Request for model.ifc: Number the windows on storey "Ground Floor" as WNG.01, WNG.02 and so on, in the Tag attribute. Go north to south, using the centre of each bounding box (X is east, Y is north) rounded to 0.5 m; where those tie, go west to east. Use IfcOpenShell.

First a look at what the model holds.

```python
import ifcopenshell
import ifcopenshell.util.element
import ifcopenshell.util.placement

model = ifcopenshell.open("model.ifc")
print(model.schema)
storey = next(s for s in model.by_type("IfcBuildingStorey") if s.Name == "Ground Floor")
windows = [e for e in ifcopenshell.util.element.get_decomposition(storey) if e.is_a("IfcWindow")]
for e in sorted(windows, key=lambda e: e.id()):
    origin = ifcopenshell.util.placement.get_local_placement(e.ObjectPlacement)[:3, 3]
    print(e.id(), e.Tag, e.Name, origin.round(2) + 0.0, sep=" | ")
```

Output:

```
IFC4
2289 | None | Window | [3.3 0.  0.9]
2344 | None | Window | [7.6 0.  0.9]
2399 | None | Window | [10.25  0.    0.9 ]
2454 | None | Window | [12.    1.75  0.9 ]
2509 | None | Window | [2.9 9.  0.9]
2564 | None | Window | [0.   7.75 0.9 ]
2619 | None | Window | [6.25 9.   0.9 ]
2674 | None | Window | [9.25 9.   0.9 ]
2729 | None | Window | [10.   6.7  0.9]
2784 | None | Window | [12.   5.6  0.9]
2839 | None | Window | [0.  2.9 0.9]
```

```python
import ifcopenshell
import ifcopenshell.geom
import ifcopenshell.util.element
import ifcopenshell.util.shape

model = ifcopenshell.open("model.ifc")
settings = ifcopenshell.geom.settings()
settings.set("use-world-coords", True)


def centre(element):
    shape = ifcopenshell.geom.create_shape(settings, element)
    return ifcopenshell.util.shape.get_bbox_centroid(shape.geometry)


storey = next(s for s in model.by_type("IfcBuildingStorey") if s.Name == "Ground Floor")
windows = [e for e in ifcopenshell.util.element.get_decomposition(storey) if e.is_a("IfcWindow")]

# Insertion points can sit at a corner or the storey origin, so sort by the geometry (in metres).
centres = {e: centre(e) for e in windows}
windows.sort(key=lambda e: (-round(centres[e][1] / 0.5), centres[e][0]))

for i, e in enumerate(windows, start=1):
    number = f"WNG.{i:02d}"
    e.Tag = number
    print(e.id(), number)

model.write("model-out.ifc")
```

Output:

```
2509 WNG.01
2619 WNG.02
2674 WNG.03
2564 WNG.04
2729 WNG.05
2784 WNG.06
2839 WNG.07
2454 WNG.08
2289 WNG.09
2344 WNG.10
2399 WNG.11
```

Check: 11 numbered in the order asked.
